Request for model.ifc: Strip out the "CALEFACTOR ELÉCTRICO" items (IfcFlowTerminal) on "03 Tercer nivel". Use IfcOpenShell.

First a look at what the model holds.

```python
import ifcopenshell
import ifcopenshell.util.element

model = ifcopenshell.open("model.ifc")
print(model.schema)
storey = next(s for s in model.by_type("IfcBuildingStorey") if s.Name == "03 Tercer nivel")
terminals = [e for e in ifcopenshell.util.element.get_decomposition(storey) if e.is_a("IfcFlowTerminal")]
seen = {}
for e in terminals:
    element_type = ifcopenshell.util.element.get_type(e)
    name = element_type.Name if element_type not in (None, e) else None
    seen[name] = seen.get(name, 0) + 1
for name, count in sorted(seen.items(), key=str):
    print(count, "x", name)
```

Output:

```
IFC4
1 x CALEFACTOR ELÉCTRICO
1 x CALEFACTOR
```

```python
import ifcopenshell
import ifcopenshell.api.root
import ifcopenshell.util.element

model = ifcopenshell.open("model.ifc")

storey = next(s for s in model.by_type("IfcBuildingStorey") if s.Name == "03 Tercer nivel")
terminals = [e for e in ifcopenshell.util.element.get_decomposition(storey) if e.is_a("IfcFlowTerminal")]
targets = [e for e in terminals if (t := ifcopenshell.util.element.get_type(e)) not in (None, e) and t.Name == "CALEFACTOR ELÉCTRICO"]

for e in targets:
    ifcopenshell.api.root.remove_product(model, product=e)
print(len(targets), "removed")

model.write("model_updated.ifc")
```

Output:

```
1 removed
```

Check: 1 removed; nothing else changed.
